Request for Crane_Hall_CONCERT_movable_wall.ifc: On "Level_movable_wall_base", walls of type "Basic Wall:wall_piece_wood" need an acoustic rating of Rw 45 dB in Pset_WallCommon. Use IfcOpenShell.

First a look at what the model holds.

```python
import ifcopenshell
import ifcopenshell.util.element

model = ifcopenshell.open("Crane_Hall_CONCERT_movable_wall.ifc")
print(model.schema)
storey = next(s for s in model.by_type("IfcBuildingStorey") if s.Name == "Level_movable_wall_base")
walls = [e for e in ifcopenshell.util.element.get_decomposition(storey) if e.is_a("IfcWall")]
seen = {}
for e in walls:
    element_type = ifcopenshell.util.element.get_type(e)
    key = (element_type.Name if element_type != e and element_type else None, ifcopenshell.util.element.get_pset(e, "Pset_WallCommon", "AcousticRating"))
    seen[key] = seen.get(key, 0) + 1
for (name, value), count in sorted(seen.items(), key=str):
    print(count, "x", name, "|", value)
```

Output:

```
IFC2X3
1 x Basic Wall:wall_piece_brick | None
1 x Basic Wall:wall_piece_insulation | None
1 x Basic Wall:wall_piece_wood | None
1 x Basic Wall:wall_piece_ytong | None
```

```python
import ifcopenshell
import ifcopenshell.api.pset
import ifcopenshell.util.element

model = ifcopenshell.open("Crane_Hall_CONCERT_movable_wall.ifc")

storey = next(s for s in model.by_type("IfcBuildingStorey") if s.Name == "Level_movable_wall_base")
walls = [e for e in ifcopenshell.util.element.get_decomposition(storey) if e.is_a("IfcWall")]

count = 0
for e in walls:
    element_type = ifcopenshell.util.element.get_type(e)
    if element_type in (None, e) or element_type.Name != "Basic Wall:wall_piece_wood":
        continue
    # add_pset returns the element's existing set when there is one.
    pset = ifcopenshell.api.pset.add_pset(model, product=e, name="Pset_WallCommon")
    ifcopenshell.api.pset.edit_pset(model, pset=pset, properties={"AcousticRating": "Rw 45 dB"})
    count += 1

print(count, "walls updated")

model.write("Crane_Hall_CONCERT_movable_wall-out.ifc")
```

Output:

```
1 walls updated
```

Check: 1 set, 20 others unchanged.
